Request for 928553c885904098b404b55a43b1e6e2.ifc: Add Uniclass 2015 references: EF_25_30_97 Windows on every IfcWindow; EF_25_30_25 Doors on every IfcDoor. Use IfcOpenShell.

First a look at what the model holds.

```python
import ifcopenshell

model = ifcopenshell.open("928553c885904098b404b55a43b1e6e2.ifc")
print(model.schema)
print("classifications:", [c.Name for c in model.by_type("IfcClassification")])
for ifc_class in ("IfcDoor", "IfcRoof", "IfcStair", "IfcWall", "IfcWindow"):
    print(ifc_class, len(model.by_type(ifc_class)))
```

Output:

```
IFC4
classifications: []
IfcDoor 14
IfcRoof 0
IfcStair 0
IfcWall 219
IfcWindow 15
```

```python
import ifcopenshell
import ifcopenshell.api.classification

model = ifcopenshell.open("928553c885904098b404b55a43b1e6e2.ifc")

system = ifcopenshell.api.classification.add_classification(model, classification="Uniclass 2015")

codes = {
    "IfcWindow": ("EF_25_30_97", "Windows"),
    "IfcDoor": ("EF_25_30_25", "Doors"),
}
for ifc_class, (code, name) in codes.items():
    products = model.by_type(ifc_class)
    ifcopenshell.api.classification.add_reference(
        model, products=products, classification=system, identification=code, name=name
    )
    print(code, len(products))

model.write("928553c885904098b404b55a43b1e6e2-out.ifc")
```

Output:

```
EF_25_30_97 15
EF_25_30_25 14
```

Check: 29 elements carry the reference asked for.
